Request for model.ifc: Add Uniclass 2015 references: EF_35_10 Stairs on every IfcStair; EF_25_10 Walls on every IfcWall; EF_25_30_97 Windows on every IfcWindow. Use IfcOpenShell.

First a look at what the model holds.

```python
import ifcopenshell

model = ifcopenshell.open("model.ifc")
print(model.schema)
print("classifications:", [c.Name for c in model.by_type("IfcClassification")])
for ifc_class in ("IfcDoor", "IfcRoof", "IfcStair", "IfcWall", "IfcWindow"):
    print(ifc_class, len(model.by_type(ifc_class)))
```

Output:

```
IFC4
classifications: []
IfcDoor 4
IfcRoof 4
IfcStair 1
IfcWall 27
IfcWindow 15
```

```python
import ifcopenshell
import ifcopenshell.api.classification

model = ifcopenshell.open("model.ifc")

system = ifcopenshell.api.classification.add_classification(model, classification="Uniclass 2015")

codes = {
    "IfcStair": ("EF_35_10", "Stairs"),
    "IfcWall": ("EF_25_10", "Walls"),
    "IfcWindow": ("EF_25_30_97", "Windows"),
}
for ifc_class, (code, name) in codes.items():
    products = model.by_type(ifc_class)
    ifcopenshell.api.classification.add_reference(
        model, products=products, classification=system, identification=code, name=name
    )
    print(code, len(products))

model.write("model-out.ifc")
```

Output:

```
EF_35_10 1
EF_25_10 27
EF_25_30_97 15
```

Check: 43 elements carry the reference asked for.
